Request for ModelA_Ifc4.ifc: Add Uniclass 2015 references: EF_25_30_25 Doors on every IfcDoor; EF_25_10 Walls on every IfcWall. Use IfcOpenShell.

First a look at what the model holds.

```python
import ifcopenshell

model = ifcopenshell.open("ModelA_Ifc4.ifc")
print(model.schema)
print("classifications:", [c.Name for c in model.by_type("IfcClassification")])
for ifc_class in ("IfcDoor", "IfcRoof", "IfcStair", "IfcWall", "IfcWindow"):
    print(ifc_class, len(model.by_type(ifc_class)))
```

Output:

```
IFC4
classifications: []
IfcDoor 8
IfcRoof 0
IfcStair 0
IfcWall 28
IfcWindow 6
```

```python
import ifcopenshell
import ifcopenshell.api.classification

model = ifcopenshell.open("ModelA_Ifc4.ifc")

system = ifcopenshell.api.classification.add_classification(model, classification="Uniclass 2015")

codes = {
    "IfcDoor": ("EF_25_30_25", "Doors"),
    "IfcWall": ("EF_25_10", "Walls"),
}
for ifc_class, (code, name) in codes.items():
    products = model.by_type(ifc_class)
    ifcopenshell.api.classification.add_reference(
        model, products=products, classification=system, identification=code, name=name
    )
    print(code, len(products))

model.write("ModelA_Ifc4_updated.ifc")
```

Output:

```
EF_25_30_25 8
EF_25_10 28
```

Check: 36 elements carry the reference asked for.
